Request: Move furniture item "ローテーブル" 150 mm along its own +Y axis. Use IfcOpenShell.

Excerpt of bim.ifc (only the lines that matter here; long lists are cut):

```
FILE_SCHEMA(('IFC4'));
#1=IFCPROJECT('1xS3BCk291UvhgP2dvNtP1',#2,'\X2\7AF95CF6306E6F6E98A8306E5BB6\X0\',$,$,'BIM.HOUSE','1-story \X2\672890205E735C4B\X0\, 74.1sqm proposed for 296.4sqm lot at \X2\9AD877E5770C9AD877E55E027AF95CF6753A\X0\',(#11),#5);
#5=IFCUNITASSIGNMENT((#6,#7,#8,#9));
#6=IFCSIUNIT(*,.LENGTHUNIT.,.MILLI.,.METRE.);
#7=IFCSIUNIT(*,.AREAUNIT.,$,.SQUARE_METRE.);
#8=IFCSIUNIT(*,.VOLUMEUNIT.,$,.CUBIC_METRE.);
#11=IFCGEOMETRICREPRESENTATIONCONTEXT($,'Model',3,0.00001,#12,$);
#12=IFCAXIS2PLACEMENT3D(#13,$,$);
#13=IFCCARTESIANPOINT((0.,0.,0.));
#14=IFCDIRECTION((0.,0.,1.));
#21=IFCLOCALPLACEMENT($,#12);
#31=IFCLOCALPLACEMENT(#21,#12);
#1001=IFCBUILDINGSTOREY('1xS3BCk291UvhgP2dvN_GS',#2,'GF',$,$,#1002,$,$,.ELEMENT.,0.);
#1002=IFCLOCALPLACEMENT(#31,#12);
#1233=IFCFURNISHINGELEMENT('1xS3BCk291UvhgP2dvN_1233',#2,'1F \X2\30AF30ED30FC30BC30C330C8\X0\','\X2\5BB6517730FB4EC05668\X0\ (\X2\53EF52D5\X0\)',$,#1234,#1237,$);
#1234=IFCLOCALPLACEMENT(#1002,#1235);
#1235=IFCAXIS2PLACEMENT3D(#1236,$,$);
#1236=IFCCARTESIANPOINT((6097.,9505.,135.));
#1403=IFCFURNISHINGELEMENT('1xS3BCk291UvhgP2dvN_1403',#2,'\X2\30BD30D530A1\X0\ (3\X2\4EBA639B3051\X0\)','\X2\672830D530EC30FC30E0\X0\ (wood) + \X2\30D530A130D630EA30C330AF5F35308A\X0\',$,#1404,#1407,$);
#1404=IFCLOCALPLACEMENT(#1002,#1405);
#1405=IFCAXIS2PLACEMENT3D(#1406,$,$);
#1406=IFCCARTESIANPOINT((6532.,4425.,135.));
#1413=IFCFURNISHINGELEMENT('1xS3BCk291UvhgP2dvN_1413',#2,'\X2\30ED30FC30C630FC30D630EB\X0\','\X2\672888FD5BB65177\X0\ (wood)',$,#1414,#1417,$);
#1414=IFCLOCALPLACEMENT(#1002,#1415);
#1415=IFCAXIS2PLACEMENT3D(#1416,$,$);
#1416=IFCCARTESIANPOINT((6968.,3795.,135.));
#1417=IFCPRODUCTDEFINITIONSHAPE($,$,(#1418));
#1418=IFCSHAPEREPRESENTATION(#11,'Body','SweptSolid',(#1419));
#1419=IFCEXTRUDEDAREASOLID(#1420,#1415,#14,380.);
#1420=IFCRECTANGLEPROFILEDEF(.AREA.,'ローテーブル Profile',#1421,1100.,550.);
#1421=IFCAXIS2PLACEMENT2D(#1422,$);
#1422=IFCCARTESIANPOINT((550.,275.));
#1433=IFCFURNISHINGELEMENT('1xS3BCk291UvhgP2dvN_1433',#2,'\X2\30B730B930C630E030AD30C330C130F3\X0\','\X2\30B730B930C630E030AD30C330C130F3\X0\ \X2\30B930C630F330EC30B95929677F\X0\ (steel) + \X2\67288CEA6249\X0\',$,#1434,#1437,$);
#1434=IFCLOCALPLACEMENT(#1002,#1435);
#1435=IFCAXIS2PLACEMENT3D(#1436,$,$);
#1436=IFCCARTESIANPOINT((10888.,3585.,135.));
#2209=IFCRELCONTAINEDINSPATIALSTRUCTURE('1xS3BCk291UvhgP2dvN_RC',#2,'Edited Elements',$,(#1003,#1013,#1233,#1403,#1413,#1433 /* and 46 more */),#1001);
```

```python
import ifcopenshell
import ifcopenshell.api.geometry
import ifcopenshell.util.placement
import ifcopenshell.util.unit

model = ifcopenshell.open("bim.ifc")
unit_scale = ifcopenshell.util.unit.calculate_unit_scale(model)

item = model.by_id(1413)
matrix = ifcopenshell.util.placement.get_local_placement(item.ObjectPlacement)
matrix[:3, 3] += matrix[:3, 1] * 0.15 / unit_scale
ifcopenshell.api.geometry.edit_object_placement(model, product=item, matrix=matrix, is_si=False)

print(ifcopenshell.util.placement.get_local_placement(item.ObjectPlacement).round(3) + 0.0)

model.write("bim_edited.ifc")
```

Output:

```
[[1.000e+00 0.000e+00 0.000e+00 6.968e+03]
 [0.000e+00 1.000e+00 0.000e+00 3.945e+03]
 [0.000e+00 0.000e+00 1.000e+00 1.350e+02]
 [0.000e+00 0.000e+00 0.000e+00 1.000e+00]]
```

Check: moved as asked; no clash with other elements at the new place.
